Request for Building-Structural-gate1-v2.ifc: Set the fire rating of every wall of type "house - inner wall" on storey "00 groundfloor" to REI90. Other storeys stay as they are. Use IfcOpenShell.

First a look at what the model holds.

```python
import ifcopenshell
import ifcopenshell.util.element

model = ifcopenshell.open("Building-Structural-gate1-v2.ifc")
print(model.schema)
storey = next(s for s in model.by_type("IfcBuildingStorey") if s.Name == "00 groundfloor")
walls = [e for e in ifcopenshell.util.element.get_decomposition(storey) if e.is_a("IfcWall")]
seen = {}
for e in walls:
    element_type = ifcopenshell.util.element.get_type(e)
    key = (element_type.Name if element_type != e and element_type else None, ifcopenshell.util.element.get_pset(e, "Pset_WallCommon", "FireRating"))
    seen[key] = seen.get(key, 0) + 1
for (name, value), count in sorted(seen.items(), key=str):
    print(count, "x", name, "|", value)
```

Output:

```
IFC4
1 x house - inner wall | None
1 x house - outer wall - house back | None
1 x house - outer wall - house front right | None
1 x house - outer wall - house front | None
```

```python
import ifcopenshell
import ifcopenshell.api.pset
import ifcopenshell.util.element

model = ifcopenshell.open("Building-Structural-gate1-v2.ifc")

storey = next(s for s in model.by_type("IfcBuildingStorey") if s.Name == "00 groundfloor")
walls = [e for e in ifcopenshell.util.element.get_decomposition(storey) if e.is_a("IfcWall")]

count = 0
for e in walls:
    element_type = ifcopenshell.util.element.get_type(e)
    if element_type in (None, e) or element_type.Name != "house - inner wall":
        continue
    # add_pset returns the element's existing set when there is one.
    pset = ifcopenshell.api.pset.add_pset(model, product=e, name="Pset_WallCommon")
    ifcopenshell.api.pset.edit_pset(model, pset=pset, properties={"FireRating": "REI90"})
    count += 1

print(count, "walls updated")

model.write("Building-Structural-gate1-v2-out.ifc")
```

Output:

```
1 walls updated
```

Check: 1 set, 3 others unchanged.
